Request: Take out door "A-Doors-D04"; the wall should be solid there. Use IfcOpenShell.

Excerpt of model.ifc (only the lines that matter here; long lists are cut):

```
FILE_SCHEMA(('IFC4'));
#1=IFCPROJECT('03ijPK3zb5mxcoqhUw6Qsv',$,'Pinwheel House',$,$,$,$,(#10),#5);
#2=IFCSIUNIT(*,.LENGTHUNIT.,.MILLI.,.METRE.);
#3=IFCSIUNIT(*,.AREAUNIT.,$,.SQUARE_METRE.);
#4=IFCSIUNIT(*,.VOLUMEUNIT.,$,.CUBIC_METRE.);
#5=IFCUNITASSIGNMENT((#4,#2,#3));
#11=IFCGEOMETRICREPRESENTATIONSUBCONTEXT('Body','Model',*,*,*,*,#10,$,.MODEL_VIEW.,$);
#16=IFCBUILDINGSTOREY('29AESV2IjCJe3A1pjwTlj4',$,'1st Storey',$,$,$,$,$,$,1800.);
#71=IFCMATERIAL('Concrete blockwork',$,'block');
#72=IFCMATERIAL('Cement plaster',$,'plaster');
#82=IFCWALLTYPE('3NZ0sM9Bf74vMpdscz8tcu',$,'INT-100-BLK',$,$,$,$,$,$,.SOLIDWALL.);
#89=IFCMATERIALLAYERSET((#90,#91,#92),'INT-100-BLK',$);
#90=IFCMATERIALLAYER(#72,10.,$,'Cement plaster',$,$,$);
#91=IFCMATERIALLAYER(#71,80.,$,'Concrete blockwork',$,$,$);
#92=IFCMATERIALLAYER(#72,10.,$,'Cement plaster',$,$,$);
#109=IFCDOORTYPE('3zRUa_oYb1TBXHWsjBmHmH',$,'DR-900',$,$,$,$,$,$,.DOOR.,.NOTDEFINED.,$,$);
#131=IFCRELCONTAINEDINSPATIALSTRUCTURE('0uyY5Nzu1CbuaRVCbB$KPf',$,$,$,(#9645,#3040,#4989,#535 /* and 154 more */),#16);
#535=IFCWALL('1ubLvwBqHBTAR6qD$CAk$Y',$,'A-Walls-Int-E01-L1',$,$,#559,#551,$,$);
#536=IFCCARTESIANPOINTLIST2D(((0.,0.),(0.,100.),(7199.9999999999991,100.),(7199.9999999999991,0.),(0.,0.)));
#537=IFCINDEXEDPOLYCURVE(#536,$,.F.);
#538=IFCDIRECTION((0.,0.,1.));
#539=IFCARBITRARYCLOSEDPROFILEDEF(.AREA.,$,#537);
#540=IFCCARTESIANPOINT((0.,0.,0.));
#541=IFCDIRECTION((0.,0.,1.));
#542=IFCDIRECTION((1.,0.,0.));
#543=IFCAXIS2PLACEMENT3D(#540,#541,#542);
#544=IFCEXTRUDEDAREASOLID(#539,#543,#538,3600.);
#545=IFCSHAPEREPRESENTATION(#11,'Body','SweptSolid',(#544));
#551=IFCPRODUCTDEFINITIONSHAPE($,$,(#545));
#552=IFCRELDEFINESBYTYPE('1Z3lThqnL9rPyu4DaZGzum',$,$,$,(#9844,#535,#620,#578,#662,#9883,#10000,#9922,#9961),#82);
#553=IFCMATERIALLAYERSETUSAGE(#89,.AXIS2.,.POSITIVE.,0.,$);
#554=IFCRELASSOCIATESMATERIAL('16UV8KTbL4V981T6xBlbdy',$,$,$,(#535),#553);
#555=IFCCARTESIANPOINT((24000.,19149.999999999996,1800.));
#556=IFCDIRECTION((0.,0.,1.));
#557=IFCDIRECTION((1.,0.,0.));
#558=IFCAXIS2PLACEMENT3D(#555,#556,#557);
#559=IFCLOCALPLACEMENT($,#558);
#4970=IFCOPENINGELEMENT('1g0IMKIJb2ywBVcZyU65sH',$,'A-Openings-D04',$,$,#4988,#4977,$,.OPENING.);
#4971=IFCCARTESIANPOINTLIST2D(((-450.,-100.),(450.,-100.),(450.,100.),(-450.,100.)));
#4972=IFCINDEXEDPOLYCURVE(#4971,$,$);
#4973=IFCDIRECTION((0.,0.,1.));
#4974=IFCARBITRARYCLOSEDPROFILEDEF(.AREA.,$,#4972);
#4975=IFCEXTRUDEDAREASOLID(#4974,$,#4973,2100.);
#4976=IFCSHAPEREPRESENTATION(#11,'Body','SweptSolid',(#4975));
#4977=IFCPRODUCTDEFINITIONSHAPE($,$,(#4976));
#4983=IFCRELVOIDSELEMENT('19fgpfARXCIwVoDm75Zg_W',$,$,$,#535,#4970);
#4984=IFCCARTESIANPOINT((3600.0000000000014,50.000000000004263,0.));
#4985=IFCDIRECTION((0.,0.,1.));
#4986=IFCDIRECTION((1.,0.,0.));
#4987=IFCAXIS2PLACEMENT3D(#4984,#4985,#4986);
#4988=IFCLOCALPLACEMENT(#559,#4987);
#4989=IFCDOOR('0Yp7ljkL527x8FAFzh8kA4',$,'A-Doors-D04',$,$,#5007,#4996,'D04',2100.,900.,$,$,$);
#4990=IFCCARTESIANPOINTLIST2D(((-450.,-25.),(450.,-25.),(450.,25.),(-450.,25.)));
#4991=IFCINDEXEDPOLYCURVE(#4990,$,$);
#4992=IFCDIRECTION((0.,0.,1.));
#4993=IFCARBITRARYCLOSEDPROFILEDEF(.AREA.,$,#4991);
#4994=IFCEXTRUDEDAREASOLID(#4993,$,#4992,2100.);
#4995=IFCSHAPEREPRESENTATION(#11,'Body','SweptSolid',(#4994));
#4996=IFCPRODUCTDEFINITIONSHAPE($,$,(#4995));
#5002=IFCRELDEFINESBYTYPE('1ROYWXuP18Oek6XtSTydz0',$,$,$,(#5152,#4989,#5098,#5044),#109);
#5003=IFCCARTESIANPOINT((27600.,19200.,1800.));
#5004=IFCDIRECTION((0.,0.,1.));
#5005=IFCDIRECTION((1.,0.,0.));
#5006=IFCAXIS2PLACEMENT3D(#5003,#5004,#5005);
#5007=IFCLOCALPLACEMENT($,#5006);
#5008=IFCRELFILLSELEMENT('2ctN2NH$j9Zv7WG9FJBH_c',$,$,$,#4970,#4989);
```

```python
import ifcopenshell
import ifcopenshell.api.feature
import ifcopenshell.api.root
import ifcopenshell.geom
import ifcopenshell.util.shape

model = ifcopenshell.open("model.ifc")
settings = ifcopenshell.geom.settings()


def volume(element):
    """Net volume in cubic metres, openings subtracted."""
    shape = ifcopenshell.geom.create_shape(settings, element)
    return ifcopenshell.util.shape.get_volume(shape.geometry)


door = model.by_id(4989)
opening = door.FillsVoids[0].RelatingOpeningElement
wall = opening.VoidsElements[0].RelatingBuildingElement
before = volume(wall)

ifcopenshell.api.root.remove_product(model, product=door)
ifcopenshell.api.feature.remove_feature(model, feature=opening)

after = volume(wall)

print(f"wall volume {before:.3f} -> {after:.3f} m3")

model.write("model_edited.ifc")
```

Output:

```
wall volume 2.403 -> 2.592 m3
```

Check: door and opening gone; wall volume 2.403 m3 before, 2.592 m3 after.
